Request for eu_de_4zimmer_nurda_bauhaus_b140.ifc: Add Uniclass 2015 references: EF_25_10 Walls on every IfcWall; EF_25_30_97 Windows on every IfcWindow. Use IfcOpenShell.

First a look at what the model holds.

```python
import ifcopenshell

model = ifcopenshell.open("eu_de_4zimmer_nurda_bauhaus_b140.ifc")
print(model.schema)
print("classifications:", [c.Name for c in model.by_type("IfcClassification")])
for ifc_class in ("IfcDoor", "IfcRoof", "IfcStair", "IfcWall", "IfcWindow"):
    print(ifc_class, len(model.by_type(ifc_class)))
```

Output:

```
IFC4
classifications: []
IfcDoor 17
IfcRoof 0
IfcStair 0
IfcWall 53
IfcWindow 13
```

```python
import ifcopenshell
import ifcopenshell.api.classification

model = ifcopenshell.open("eu_de_4zimmer_nurda_bauhaus_b140.ifc")

system = ifcopenshell.api.classification.add_classification(model, classification="Uniclass 2015")

codes = {
    "IfcWall": ("EF_25_10", "Walls"),
    "IfcWindow": ("EF_25_30_97", "Windows"),
}
for ifc_class, (code, name) in codes.items():
    products = model.by_type(ifc_class)
    ifcopenshell.api.classification.add_reference(
        model, products=products, classification=system, identification=code, name=name
    )
    print(code, len(products))

model.write("eu_de_4zimmer_nurda_bauhaus_b140_updated.ifc")
```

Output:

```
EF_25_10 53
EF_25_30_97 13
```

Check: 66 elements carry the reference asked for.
